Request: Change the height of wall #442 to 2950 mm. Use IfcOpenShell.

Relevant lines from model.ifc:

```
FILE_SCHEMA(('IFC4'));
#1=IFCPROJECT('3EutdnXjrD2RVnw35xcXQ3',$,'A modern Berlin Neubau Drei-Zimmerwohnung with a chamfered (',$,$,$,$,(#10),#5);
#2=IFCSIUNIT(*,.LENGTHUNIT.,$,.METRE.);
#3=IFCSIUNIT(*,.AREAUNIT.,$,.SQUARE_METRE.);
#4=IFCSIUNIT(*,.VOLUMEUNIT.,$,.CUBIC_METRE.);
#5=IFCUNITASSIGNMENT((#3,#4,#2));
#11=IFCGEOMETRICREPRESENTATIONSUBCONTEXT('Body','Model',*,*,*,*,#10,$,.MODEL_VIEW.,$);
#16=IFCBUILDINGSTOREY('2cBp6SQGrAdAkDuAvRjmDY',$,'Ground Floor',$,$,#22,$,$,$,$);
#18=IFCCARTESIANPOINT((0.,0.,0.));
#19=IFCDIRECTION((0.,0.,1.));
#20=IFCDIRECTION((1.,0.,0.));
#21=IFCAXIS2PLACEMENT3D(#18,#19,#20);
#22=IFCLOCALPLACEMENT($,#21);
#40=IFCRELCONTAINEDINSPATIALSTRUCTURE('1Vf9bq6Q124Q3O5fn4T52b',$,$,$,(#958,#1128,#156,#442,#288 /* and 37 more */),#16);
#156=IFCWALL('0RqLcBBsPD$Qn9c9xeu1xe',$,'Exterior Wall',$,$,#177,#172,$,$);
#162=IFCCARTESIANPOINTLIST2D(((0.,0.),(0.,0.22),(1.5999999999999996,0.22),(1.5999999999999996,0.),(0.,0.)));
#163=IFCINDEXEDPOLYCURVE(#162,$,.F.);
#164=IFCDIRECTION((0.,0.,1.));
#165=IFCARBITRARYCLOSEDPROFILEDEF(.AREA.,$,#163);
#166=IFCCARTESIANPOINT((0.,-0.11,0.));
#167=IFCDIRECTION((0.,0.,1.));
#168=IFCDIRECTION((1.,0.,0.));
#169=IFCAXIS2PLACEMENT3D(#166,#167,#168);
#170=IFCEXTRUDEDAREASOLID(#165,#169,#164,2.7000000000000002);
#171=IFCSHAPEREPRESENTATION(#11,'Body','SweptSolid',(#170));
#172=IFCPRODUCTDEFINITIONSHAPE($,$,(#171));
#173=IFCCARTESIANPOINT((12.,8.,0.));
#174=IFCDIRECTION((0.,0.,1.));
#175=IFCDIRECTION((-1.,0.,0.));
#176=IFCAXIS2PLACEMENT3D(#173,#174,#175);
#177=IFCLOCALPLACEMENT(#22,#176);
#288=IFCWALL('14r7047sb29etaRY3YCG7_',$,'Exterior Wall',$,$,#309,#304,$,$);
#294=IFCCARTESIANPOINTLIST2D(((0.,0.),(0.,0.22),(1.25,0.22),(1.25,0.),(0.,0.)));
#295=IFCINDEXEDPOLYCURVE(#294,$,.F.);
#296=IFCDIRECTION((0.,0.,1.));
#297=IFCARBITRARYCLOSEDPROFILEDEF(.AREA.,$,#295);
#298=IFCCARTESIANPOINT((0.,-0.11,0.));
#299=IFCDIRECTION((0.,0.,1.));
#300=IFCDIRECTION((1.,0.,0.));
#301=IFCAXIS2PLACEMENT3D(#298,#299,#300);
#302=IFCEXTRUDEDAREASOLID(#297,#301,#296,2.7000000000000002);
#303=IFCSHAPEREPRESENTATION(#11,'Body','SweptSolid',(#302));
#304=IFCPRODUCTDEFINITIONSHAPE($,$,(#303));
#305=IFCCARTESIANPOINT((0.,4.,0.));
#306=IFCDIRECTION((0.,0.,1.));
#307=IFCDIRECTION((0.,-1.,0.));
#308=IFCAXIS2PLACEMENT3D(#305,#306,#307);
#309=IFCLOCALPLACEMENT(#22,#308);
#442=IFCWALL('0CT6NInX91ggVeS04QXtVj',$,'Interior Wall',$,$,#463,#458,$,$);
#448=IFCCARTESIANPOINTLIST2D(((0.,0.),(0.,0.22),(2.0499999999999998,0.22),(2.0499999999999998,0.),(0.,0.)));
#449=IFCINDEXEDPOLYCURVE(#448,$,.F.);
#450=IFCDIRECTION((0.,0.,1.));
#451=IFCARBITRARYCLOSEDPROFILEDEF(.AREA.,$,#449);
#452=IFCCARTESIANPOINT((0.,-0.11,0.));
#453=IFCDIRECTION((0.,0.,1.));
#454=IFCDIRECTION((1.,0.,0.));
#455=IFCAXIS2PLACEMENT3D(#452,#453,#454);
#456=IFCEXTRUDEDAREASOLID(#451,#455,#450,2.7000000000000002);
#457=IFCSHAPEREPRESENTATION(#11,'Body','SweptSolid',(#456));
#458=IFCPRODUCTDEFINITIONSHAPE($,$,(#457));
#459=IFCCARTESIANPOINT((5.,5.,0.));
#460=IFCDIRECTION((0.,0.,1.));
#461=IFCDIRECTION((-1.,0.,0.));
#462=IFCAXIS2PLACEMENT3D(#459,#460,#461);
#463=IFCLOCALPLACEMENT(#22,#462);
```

```python
import ifcopenshell
import ifcopenshell.geom
import ifcopenshell.util.representation
import ifcopenshell.util.shape
import ifcopenshell.util.unit

model = ifcopenshell.open("model.ifc")
unit_scale = ifcopenshell.util.unit.calculate_unit_scale(model)
settings = ifcopenshell.geom.settings()


def volume(element):
    """Net volume in cubic metres, openings subtracted."""
    shape = ifcopenshell.geom.create_shape(settings, element)
    return ifcopenshell.util.shape.get_volume(shape.geometry)


wall = model.by_guid("0CT6NInX91ggVeS04QXtVj")
before = volume(wall)

body = ifcopenshell.util.representation.get_representation(wall, "Model", "Body")
solid = body.Items[0]
old_height = solid.Depth
solid.Depth = 2.95 / unit_scale
after = volume(wall)

print(f"height {old_height:g} -> {solid.Depth:g}, volume {before:.3f} -> {after:.3f} m3")

model.write("model_v2.ifc")
```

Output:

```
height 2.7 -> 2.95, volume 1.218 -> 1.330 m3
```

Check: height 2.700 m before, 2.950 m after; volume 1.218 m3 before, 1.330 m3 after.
